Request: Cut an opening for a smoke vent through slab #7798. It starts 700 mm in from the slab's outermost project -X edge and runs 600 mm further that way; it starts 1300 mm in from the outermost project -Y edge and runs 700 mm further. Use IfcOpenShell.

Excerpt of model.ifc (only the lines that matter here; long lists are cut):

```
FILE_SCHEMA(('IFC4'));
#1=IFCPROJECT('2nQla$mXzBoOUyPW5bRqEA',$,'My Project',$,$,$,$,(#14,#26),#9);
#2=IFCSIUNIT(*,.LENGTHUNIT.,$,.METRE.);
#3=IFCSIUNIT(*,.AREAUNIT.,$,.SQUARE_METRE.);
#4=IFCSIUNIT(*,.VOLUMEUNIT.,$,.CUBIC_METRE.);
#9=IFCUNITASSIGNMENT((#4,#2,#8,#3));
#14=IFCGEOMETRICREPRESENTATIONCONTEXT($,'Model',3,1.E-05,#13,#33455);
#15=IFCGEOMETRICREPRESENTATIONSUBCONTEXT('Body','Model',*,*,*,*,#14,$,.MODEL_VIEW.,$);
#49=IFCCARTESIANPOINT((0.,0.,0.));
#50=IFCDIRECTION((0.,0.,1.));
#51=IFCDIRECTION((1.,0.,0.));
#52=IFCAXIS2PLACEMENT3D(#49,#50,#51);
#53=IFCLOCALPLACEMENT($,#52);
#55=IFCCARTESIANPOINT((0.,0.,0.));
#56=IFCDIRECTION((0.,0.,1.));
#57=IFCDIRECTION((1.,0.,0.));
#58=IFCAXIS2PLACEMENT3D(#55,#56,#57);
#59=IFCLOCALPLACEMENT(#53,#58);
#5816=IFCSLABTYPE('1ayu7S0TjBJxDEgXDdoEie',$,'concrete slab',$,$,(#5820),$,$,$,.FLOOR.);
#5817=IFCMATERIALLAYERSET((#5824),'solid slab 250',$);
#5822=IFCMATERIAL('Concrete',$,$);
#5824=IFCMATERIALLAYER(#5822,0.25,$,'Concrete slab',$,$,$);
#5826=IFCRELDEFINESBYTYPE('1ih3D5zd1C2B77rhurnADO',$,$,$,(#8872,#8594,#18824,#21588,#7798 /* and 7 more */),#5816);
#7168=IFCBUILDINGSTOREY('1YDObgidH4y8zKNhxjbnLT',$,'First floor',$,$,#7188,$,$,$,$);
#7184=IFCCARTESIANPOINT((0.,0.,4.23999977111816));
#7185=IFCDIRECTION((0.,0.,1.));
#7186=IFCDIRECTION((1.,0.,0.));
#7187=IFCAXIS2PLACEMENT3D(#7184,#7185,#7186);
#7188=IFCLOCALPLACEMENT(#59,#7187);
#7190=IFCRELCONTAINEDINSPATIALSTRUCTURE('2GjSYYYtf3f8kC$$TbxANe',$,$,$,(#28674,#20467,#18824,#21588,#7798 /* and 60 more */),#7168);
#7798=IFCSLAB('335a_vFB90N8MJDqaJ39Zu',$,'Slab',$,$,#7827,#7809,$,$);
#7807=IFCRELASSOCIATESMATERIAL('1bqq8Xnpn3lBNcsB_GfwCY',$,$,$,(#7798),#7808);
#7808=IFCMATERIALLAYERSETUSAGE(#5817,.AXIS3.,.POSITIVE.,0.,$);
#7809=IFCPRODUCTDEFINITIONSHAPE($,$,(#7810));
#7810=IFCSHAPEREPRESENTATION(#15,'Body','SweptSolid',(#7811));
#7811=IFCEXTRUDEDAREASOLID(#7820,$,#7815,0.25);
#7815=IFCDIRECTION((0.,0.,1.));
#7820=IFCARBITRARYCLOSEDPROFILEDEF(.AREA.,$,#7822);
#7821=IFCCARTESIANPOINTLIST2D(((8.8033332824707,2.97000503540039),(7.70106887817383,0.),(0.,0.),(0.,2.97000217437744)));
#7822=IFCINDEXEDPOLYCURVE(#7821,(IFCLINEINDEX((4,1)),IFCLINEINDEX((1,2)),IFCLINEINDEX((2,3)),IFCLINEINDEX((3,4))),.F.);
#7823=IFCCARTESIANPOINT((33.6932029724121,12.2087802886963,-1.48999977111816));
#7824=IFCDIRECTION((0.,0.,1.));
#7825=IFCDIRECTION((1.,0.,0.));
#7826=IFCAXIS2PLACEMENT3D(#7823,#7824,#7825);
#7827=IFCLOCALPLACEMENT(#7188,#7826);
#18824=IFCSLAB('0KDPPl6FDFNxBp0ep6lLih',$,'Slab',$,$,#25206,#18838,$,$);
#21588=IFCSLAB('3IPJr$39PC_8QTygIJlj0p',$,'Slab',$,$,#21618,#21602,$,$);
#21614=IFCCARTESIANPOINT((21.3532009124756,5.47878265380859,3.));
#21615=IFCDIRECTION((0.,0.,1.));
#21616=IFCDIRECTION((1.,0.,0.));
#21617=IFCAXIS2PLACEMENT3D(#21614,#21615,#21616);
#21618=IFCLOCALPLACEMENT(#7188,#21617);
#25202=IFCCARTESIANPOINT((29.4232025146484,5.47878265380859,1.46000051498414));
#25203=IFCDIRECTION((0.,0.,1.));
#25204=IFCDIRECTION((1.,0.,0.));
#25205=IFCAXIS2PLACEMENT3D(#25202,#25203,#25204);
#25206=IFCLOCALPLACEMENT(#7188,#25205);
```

```python
import numpy as np
import ifcopenshell
import ifcopenshell.api.feature
import ifcopenshell.api.geometry
import ifcopenshell.api.root
import ifcopenshell.geom
import ifcopenshell.util.placement
import ifcopenshell.util.representation
import ifcopenshell.util.shape
import ifcopenshell.util.unit

model = ifcopenshell.open("model.ifc")
unit_scale = ifcopenshell.util.unit.calculate_unit_scale(model)
settings = ifcopenshell.geom.settings()


def volume(element):
    """Net volume in cubic metres, openings subtracted."""
    shape = ifcopenshell.geom.create_shape(settings, element)
    return ifcopenshell.util.shape.get_volume(shape.geometry)


slab = model.by_id(7798)
before = volume(slab)

# Extent in the slab's own axes, in metres. The edges named are its -X and -Y sides.
slab_shape = ifcopenshell.geom.create_shape(settings, slab)
vertices = ifcopenshell.util.shape.get_vertices(slab_shape.geometry)
x_min, y_min, bottom = vertices.min(axis=0)
top = vertices[:, 2].max()

opening = ifcopenshell.api.root.create_entity(model, ifc_class="IfcOpeningElement", name="Smoke vent opening", predefined_type="OPENING")
context = ifcopenshell.util.representation.get_context(model, "Model", "Body", "MODEL_VIEW")
width, depth = 0.6, 0.7
outline = [(0.0, 0.0), (width, 0.0), (width, depth), (0.0, depth), (0.0, 0.0)]
# Overshoot both faces by 50 mm so the cut is clean.
shape = ifcopenshell.api.geometry.add_slab_representation(
    model, context=context, depth=top - bottom + 0.1, polyline=outline
)
ifcopenshell.api.geometry.assign_representation(model, product=opening, representation=shape)

matrix = ifcopenshell.util.placement.get_local_placement(slab.ObjectPlacement)
matrix[:, 3] = matrix @ np.append(np.array([x_min + 0.7, y_min + 1.3, bottom - 0.05]) / unit_scale, 1.0)
ifcopenshell.api.geometry.edit_object_placement(model, product=opening, matrix=matrix, is_si=False)
ifcopenshell.api.feature.add_feature(model, feature=opening, element=slab)

after = volume(slab)

print(f"slab volume {before:.3f} -> {after:.3f} m3")

model.write("model_v2.ifc")
```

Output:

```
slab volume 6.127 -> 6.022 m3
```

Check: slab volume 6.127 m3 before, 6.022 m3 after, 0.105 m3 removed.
